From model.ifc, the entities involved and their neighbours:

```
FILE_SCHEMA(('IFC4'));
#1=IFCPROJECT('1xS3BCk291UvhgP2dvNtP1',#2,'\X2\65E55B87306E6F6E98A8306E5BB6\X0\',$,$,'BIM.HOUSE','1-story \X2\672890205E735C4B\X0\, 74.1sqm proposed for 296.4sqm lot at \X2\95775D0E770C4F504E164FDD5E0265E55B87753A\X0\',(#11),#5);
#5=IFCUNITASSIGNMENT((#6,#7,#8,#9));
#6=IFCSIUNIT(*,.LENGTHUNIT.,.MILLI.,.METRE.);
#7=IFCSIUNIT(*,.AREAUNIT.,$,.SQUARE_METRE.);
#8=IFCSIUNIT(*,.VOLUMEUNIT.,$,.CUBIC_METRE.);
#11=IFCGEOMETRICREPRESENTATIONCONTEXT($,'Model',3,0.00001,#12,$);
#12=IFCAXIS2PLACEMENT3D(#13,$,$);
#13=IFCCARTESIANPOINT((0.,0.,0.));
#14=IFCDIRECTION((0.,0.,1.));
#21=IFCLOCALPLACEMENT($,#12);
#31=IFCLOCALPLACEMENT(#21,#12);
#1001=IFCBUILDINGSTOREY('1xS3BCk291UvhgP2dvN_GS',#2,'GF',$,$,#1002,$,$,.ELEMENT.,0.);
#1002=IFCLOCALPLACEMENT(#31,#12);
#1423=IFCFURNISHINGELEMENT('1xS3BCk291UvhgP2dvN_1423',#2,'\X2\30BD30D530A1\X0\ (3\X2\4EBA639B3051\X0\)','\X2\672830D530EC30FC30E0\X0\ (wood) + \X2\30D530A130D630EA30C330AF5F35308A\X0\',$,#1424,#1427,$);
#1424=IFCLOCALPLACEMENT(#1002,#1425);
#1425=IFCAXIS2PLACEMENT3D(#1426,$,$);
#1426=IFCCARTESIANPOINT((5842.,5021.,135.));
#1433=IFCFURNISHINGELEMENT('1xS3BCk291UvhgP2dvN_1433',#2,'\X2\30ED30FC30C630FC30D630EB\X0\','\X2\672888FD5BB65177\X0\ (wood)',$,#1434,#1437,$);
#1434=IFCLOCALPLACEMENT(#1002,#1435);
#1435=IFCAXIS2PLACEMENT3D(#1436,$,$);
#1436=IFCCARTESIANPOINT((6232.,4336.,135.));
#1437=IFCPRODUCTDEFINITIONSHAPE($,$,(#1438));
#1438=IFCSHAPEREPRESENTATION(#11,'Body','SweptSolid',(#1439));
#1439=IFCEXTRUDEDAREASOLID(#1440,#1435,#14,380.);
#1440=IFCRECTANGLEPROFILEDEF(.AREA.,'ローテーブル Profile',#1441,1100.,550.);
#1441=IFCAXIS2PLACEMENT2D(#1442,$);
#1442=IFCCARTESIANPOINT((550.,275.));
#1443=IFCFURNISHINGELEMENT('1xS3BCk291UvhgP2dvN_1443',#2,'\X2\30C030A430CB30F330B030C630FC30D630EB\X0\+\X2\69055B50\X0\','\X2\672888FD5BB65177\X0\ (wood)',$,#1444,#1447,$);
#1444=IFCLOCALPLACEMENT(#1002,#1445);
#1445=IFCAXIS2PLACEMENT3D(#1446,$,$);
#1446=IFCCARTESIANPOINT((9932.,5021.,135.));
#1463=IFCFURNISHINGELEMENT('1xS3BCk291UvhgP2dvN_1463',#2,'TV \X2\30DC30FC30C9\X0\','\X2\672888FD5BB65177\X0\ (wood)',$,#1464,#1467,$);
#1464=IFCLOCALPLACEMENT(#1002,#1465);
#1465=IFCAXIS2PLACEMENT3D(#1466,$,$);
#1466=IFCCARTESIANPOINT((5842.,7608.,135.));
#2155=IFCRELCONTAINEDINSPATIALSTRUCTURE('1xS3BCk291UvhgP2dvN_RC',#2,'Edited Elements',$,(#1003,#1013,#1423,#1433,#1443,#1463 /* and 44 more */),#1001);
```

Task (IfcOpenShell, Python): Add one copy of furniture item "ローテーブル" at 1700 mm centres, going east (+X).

```python
import numpy as np
import ifcopenshell
import ifcopenshell.api.geometry
import ifcopenshell.api.root
import ifcopenshell.util.element
import ifcopenshell.util.placement
import ifcopenshell.util.unit

model = ifcopenshell.open("model.ifc")
unit_scale = ifcopenshell.util.unit.calculate_unit_scale(model)


def reuse_history(source, copy):
    """copy_class also copies each property set's owner history, people and application; keep the originals."""
    for rel in copy.IsDefinedBy:
        if rel.is_a("IfcRelDefinesByProperties") and (history := rel.RelatingPropertyDefinition.OwnerHistory):
            rel.RelatingPropertyDefinition.OwnerHistory = source.OwnerHistory
            ifcopenshell.util.element.remove_deep2(model, history)


source = model.by_guid("1xS3BCk291UvhgP2dvN_1433")
base = ifcopenshell.util.placement.get_local_placement(source.ObjectPlacement)
step = np.array([1.0, 0.0, 0.0]) * 1.7 / unit_scale

for i in range(1, 2):
    copy = ifcopenshell.api.root.copy_class(model, product=source)
    copy.Representation = ifcopenshell.util.element.copy_deep(
        model, source.Representation, exclude=["IfcGeometricRepresentationContext", "IfcRepresentationMap"]
    )
    reuse_history(source, copy)
    matrix = base.copy()
    matrix[:3, 3] += i * step
    print("added at", matrix[:3, 3].round(3) + 0.0)
    ifcopenshell.api.geometry.edit_object_placement(model, product=copy, matrix=matrix, is_si=False)

model.write("model_rev.ifc")
```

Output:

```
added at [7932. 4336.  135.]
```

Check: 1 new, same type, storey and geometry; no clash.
